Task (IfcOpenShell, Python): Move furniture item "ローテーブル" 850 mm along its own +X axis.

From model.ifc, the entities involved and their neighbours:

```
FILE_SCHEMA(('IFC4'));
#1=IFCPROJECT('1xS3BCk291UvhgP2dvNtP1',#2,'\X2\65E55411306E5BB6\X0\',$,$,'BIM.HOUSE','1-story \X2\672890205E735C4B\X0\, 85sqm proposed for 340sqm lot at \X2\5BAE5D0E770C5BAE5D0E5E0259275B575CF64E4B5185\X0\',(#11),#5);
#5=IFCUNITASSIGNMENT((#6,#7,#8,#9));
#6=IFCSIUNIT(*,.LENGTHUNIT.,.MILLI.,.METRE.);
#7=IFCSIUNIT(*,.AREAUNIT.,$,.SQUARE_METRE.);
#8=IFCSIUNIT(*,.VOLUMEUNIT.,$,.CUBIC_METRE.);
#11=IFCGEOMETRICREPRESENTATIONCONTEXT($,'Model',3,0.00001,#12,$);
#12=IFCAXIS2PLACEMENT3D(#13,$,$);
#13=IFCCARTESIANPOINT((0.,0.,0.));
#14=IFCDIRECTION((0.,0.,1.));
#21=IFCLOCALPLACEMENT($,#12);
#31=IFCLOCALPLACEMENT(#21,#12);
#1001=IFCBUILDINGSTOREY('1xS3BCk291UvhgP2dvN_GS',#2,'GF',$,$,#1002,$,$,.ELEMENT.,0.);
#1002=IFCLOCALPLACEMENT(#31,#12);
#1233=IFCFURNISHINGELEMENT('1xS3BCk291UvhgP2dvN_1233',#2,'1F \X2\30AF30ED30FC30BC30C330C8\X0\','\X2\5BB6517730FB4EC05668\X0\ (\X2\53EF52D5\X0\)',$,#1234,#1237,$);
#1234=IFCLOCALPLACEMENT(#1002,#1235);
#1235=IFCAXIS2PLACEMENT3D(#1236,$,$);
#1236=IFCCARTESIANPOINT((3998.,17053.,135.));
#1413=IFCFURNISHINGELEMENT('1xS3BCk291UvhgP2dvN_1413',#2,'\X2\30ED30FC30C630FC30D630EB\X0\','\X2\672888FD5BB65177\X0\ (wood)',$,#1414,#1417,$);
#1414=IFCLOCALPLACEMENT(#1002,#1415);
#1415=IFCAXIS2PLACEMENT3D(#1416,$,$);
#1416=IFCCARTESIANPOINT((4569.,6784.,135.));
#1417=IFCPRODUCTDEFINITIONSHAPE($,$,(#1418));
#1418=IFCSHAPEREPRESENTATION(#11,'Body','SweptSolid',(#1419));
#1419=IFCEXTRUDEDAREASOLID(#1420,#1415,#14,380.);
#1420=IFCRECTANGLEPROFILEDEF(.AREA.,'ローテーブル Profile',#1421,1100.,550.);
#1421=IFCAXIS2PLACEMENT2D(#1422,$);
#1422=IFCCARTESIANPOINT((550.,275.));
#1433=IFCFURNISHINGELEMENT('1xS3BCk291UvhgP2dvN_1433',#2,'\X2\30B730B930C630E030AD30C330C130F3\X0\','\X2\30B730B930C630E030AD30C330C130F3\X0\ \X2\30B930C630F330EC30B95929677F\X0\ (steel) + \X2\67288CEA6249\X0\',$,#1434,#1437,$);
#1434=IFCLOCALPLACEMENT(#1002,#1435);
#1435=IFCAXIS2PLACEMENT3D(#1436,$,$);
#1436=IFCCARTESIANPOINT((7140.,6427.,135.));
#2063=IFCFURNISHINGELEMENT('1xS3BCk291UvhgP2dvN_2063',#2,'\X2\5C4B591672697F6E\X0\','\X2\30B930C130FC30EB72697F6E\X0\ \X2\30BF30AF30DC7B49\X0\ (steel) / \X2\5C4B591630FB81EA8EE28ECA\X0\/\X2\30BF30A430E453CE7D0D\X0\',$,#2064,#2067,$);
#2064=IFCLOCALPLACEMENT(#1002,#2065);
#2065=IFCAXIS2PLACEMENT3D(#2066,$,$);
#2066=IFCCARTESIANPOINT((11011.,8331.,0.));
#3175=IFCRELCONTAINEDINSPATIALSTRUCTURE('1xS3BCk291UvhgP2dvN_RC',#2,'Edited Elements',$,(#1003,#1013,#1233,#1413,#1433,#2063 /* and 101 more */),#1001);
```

```python
import ifcopenshell
import ifcopenshell.api.geometry
import ifcopenshell.util.placement

model = ifcopenshell.open("model.ifc")

item = model.by_id(1413)
matrix = ifcopenshell.util.placement.get_local_placement(item.ObjectPlacement)
matrix[:3, 3] += matrix[:3, 0] * 850.0
ifcopenshell.api.geometry.edit_object_placement(model, product=item, matrix=matrix, is_si=False)

print(ifcopenshell.util.placement.get_local_placement(item.ObjectPlacement).round(3) + 0.0)

model.write("model_edited.ifc")
```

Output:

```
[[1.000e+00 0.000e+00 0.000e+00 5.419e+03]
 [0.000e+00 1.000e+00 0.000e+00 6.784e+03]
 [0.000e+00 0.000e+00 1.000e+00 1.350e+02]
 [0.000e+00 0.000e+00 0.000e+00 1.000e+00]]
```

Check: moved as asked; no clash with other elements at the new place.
